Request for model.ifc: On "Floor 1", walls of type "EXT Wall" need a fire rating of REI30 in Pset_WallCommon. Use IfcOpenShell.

First a look at what the model holds.

```python
import ifcopenshell
import ifcopenshell.util.element

model = ifcopenshell.open("model.ifc")
print(model.schema)
storey = next(s for s in model.by_type("IfcBuildingStorey") if s.Name == "Floor 1")
walls = [e for e in ifcopenshell.util.element.get_decomposition(storey) if e.is_a("IfcWall")]
seen = {}
for e in walls:
    element_type = ifcopenshell.util.element.get_type(e)
    key = (element_type.Name if element_type != e and element_type else None, ifcopenshell.util.element.get_pset(e, "Pset_WallCommon", "FireRating"))
    seen[key] = seen.get(key, 0) + 1
for (name, value), count in sorted(seen.items(), key=str):
    print(count, "x", name, "|", value)
```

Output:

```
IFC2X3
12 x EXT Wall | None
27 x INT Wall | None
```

```python
import ifcopenshell
import ifcopenshell.api.pset
import ifcopenshell.util.element

model = ifcopenshell.open("model.ifc")

storey = next(s for s in model.by_type("IfcBuildingStorey") if s.Name == "Floor 1")
walls = [e for e in ifcopenshell.util.element.get_decomposition(storey) if e.is_a("IfcWall")]

count = 0
for e in walls:
    element_type = ifcopenshell.util.element.get_type(e)
    if element_type in (None, e) or element_type.Name != "EXT Wall":
        continue
    # add_pset returns the element's existing set when there is one.
    pset = ifcopenshell.api.pset.add_pset(model, product=e, name="Pset_WallCommon")
    ifcopenshell.api.pset.edit_pset(model, pset=pset, properties={"FireRating": "REI30"})
    count += 1

print(count, "walls updated")

model.write("model_updated.ifc")
```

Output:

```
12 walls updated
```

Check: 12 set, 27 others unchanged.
